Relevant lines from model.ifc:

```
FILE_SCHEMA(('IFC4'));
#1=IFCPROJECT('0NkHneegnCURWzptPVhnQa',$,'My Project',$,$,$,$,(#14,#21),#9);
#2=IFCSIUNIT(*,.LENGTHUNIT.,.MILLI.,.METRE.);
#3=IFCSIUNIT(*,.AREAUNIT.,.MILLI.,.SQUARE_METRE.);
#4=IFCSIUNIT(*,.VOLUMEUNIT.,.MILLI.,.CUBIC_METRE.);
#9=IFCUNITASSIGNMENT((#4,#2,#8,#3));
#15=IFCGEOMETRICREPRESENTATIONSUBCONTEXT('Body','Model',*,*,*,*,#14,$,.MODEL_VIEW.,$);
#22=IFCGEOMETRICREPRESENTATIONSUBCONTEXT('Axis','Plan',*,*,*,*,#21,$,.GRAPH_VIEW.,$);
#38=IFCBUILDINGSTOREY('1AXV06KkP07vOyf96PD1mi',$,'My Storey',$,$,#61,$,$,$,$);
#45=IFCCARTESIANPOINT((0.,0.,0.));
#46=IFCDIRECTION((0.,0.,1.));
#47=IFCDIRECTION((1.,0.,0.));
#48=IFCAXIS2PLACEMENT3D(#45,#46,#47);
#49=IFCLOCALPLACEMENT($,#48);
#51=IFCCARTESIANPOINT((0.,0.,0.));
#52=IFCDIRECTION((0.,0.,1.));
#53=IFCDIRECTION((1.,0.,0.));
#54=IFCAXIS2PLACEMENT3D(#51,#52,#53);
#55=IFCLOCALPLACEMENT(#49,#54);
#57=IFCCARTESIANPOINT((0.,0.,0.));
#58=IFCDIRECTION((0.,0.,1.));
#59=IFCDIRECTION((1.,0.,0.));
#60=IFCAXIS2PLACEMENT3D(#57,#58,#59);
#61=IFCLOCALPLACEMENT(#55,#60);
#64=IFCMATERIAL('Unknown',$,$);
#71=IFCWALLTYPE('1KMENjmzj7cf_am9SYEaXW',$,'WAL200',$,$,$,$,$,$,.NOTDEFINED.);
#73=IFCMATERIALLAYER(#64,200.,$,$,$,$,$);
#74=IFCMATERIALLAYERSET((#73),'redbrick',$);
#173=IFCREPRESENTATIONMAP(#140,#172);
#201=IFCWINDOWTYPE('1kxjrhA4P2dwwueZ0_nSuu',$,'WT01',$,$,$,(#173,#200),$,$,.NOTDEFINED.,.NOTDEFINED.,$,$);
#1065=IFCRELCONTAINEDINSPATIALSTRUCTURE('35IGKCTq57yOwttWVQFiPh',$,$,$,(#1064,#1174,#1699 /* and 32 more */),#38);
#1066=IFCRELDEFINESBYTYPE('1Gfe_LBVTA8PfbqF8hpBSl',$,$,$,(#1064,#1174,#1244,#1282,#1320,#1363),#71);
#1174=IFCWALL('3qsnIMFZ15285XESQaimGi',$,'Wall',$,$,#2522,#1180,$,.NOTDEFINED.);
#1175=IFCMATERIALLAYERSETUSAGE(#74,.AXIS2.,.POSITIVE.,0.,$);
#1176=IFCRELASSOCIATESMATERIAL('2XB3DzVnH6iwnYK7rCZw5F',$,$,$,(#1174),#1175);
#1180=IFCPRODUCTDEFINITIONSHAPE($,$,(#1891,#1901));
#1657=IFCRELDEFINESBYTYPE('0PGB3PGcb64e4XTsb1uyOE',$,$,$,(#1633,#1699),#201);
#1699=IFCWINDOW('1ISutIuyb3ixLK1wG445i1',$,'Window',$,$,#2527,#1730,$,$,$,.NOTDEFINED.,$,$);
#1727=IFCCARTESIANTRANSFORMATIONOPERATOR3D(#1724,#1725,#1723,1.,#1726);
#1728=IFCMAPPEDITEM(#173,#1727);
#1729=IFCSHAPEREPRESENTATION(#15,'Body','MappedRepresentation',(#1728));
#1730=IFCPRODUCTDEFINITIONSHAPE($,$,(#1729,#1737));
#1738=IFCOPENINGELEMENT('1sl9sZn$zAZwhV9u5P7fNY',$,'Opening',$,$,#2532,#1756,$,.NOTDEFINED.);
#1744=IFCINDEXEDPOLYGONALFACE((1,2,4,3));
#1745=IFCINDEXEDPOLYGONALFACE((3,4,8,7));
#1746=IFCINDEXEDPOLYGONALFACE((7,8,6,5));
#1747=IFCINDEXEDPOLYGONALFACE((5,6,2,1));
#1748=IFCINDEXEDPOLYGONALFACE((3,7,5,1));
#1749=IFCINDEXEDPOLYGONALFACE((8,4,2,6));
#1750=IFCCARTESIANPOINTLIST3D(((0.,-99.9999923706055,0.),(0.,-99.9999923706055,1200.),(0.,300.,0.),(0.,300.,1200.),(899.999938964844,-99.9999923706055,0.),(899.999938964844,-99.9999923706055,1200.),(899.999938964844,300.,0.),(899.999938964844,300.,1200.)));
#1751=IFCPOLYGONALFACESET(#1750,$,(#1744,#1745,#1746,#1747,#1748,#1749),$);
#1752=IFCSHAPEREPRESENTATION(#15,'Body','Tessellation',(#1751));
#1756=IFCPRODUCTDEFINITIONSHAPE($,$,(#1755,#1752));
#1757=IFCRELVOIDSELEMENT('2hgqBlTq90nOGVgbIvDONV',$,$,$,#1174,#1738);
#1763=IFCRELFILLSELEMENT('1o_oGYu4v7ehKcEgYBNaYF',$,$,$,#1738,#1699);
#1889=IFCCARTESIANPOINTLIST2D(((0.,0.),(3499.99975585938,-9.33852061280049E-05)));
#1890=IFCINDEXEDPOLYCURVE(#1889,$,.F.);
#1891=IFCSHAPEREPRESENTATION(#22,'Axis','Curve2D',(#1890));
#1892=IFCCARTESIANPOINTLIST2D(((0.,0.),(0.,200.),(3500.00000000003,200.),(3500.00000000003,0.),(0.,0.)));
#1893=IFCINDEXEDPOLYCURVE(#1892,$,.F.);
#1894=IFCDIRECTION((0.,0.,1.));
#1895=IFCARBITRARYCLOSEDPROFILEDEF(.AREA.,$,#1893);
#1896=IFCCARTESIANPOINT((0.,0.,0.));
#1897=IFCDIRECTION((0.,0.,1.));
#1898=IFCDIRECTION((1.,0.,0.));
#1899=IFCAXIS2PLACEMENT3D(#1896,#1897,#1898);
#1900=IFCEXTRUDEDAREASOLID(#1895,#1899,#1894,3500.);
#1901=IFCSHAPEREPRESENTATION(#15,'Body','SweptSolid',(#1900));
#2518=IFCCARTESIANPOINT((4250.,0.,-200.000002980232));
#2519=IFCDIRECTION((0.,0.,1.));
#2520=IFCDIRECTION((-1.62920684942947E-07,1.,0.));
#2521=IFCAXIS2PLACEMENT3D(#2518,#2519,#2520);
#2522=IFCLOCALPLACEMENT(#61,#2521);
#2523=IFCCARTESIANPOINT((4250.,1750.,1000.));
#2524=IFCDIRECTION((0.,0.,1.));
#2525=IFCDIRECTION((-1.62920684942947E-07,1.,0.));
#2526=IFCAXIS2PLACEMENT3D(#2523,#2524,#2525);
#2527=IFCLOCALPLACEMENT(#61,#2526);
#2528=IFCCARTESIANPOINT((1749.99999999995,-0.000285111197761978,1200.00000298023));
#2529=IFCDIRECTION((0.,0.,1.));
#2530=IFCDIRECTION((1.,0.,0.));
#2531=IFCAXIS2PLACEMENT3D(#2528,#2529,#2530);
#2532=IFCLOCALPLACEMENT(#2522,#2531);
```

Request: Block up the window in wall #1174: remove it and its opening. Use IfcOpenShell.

```python
import ifcopenshell
import ifcopenshell.api.feature
import ifcopenshell.api.root
import ifcopenshell.geom
import ifcopenshell.util.shape

model = ifcopenshell.open("model.ifc")
settings = ifcopenshell.geom.settings()


def volume(element):
    """Net volume in cubic metres, openings subtracted."""
    shape = ifcopenshell.geom.create_shape(settings, element)
    return ifcopenshell.util.shape.get_volume(shape.geometry)


window = model.by_guid("1ISutIuyb3ixLK1wG445i1")
opening = window.FillsVoids[0].RelatingOpeningElement
wall = opening.VoidsElements[0].RelatingBuildingElement
before = volume(wall)

ifcopenshell.api.root.remove_product(model, product=window)
ifcopenshell.api.feature.remove_feature(model, feature=opening)

after = volume(wall)

print(f"wall volume {before:.3f} -> {after:.3f} m3")

model.write("model_rev.ifc")
```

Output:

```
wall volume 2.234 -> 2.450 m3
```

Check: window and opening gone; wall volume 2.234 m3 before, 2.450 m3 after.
